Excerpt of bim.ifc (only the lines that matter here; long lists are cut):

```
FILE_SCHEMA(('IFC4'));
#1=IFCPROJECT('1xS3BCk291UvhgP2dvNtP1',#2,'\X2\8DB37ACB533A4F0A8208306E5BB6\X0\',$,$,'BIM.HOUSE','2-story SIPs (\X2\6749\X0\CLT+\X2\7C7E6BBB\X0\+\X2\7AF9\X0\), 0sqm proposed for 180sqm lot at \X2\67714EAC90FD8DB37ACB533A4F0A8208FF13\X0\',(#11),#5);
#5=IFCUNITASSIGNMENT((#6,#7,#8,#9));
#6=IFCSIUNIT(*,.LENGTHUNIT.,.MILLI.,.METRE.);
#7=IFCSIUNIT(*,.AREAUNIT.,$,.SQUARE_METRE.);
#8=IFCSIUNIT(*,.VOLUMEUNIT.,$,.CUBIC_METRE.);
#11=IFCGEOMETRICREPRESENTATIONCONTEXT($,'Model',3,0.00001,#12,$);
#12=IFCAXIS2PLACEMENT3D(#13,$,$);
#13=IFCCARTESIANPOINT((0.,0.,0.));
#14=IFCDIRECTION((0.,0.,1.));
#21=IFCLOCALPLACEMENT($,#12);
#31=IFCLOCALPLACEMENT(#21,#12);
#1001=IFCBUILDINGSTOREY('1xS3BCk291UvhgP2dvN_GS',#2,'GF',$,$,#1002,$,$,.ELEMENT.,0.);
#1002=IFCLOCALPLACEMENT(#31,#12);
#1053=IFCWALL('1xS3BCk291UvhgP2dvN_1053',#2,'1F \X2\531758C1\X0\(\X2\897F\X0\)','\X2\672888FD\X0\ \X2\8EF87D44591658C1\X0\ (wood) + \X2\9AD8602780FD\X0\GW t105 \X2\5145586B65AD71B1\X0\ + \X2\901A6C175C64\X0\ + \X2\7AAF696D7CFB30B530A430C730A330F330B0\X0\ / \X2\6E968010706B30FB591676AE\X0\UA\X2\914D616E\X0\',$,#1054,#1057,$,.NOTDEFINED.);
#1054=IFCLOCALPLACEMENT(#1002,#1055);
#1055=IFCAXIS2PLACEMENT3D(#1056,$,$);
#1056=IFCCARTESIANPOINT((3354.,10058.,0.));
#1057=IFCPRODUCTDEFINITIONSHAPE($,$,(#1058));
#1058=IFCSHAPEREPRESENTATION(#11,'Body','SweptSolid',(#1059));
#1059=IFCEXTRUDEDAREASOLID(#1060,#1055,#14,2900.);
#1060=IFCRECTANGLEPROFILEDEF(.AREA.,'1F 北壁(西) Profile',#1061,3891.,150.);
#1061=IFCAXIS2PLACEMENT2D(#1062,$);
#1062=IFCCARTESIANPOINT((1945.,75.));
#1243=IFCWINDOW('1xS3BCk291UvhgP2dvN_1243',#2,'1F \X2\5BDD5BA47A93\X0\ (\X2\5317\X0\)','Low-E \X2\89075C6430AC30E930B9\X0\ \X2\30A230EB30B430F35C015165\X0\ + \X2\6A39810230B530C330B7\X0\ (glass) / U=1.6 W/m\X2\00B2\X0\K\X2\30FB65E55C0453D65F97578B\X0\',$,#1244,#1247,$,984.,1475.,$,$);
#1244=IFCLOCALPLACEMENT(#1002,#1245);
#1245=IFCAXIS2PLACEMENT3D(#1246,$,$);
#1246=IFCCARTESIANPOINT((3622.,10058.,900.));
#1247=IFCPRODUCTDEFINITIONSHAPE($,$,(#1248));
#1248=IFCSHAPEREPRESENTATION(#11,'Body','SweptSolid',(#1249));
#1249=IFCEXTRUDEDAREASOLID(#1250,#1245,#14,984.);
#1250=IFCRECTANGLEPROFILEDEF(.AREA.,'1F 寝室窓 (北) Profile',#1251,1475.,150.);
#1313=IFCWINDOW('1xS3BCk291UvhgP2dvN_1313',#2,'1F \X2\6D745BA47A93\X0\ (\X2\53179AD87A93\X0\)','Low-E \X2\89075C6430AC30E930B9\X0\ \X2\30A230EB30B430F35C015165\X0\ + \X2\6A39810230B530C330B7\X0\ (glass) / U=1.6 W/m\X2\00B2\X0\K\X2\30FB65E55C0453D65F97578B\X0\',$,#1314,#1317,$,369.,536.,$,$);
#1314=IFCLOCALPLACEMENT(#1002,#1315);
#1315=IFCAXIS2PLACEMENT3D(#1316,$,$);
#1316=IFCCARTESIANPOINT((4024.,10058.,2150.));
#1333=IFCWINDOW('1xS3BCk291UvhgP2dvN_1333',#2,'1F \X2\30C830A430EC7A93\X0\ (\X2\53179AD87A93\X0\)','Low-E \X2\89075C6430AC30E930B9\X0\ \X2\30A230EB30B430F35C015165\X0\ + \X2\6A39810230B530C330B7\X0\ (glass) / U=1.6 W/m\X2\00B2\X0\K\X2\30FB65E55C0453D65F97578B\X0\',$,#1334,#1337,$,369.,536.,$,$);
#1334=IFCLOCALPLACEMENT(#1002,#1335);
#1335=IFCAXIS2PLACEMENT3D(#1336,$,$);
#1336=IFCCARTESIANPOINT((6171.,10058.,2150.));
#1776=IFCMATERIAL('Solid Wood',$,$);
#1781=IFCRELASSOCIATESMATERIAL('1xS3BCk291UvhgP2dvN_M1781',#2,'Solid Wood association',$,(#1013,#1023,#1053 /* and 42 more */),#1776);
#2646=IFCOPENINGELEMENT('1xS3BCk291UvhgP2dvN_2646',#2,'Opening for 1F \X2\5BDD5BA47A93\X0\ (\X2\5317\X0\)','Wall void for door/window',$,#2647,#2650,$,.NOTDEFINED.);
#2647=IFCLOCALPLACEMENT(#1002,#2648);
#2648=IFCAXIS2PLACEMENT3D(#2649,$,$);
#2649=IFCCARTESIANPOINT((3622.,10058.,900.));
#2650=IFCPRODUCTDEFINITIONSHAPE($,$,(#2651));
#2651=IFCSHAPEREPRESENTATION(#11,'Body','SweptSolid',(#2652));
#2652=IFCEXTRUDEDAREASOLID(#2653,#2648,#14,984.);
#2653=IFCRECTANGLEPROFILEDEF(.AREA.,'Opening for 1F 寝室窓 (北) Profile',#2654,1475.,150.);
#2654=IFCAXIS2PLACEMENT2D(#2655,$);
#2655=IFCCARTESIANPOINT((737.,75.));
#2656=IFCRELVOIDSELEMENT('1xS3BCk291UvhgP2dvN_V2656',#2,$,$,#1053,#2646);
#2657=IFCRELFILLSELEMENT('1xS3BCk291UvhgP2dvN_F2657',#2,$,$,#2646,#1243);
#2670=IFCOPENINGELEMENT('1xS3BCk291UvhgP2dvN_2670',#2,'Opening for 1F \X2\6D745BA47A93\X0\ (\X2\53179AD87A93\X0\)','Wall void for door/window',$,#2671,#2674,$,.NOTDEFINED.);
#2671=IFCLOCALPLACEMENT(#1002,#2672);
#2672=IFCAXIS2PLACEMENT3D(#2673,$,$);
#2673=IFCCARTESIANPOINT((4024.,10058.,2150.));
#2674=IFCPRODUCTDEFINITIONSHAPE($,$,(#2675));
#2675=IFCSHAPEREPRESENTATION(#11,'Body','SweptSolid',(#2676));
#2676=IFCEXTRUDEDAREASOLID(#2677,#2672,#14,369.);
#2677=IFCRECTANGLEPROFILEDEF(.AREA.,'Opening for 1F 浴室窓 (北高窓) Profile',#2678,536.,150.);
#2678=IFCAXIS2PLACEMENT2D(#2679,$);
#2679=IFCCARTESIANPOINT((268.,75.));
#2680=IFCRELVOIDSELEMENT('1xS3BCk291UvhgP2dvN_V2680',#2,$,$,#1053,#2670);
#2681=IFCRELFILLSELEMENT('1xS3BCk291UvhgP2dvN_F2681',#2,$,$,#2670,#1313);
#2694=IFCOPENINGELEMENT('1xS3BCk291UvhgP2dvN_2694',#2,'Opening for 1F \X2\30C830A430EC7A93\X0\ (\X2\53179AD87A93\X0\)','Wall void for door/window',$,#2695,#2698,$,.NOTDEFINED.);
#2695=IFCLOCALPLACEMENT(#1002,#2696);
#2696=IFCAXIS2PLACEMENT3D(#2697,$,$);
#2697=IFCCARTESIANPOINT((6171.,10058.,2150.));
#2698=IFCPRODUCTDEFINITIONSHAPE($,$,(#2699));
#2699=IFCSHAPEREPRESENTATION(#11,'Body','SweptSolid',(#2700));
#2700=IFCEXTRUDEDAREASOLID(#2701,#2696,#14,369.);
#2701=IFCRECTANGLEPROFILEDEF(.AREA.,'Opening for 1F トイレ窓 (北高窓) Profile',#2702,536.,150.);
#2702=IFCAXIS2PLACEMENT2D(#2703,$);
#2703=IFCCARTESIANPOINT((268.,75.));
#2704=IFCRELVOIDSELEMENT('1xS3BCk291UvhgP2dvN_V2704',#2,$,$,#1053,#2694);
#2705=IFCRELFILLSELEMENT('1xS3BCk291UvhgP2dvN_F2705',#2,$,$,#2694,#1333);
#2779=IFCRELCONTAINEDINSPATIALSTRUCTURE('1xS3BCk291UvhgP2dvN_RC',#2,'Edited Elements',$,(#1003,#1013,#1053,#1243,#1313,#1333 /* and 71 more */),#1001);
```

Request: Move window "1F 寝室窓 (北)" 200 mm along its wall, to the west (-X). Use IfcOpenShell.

```python
import ifcopenshell
import ifcopenshell.api.geometry
import ifcopenshell.util.placement
import ifcopenshell.util.unit

model = ifcopenshell.open("bim.ifc")
unit_scale = ifcopenshell.util.unit.calculate_unit_scale(model)

window = model.by_guid("1xS3BCk291UvhgP2dvN_1243")
opening = window.FillsVoids[0].RelatingOpeningElement
wall = opening.VoidsElements[0].RelatingBuildingElement

wall_matrix = ifcopenshell.util.placement.get_local_placement(wall.ObjectPlacement)
shift = wall_matrix[:3, 0] * -0.2 / unit_scale
before = ifcopenshell.util.placement.get_local_placement(window.ObjectPlacement)[:3, 3].copy()

# The window is not placed relative to its opening, so move both.
for product in (opening, window):
    matrix = ifcopenshell.util.placement.get_local_placement(product.ObjectPlacement)
    matrix[:3, 3] += shift
    ifcopenshell.api.geometry.edit_object_placement(model, product=product, matrix=matrix, is_si=False)

after = ifcopenshell.util.placement.get_local_placement(window.ObjectPlacement)[:3, 3]
print("window moved by", (after - before).round(3) + 0.0)

model.write("bim_rev.ifc")
```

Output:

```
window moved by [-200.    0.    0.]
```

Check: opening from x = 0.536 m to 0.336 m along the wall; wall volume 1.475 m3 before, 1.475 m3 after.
